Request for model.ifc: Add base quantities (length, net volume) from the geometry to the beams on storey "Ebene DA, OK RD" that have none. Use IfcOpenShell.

First a look at what the model holds.

```python
import ifcopenshell
import ifcopenshell.util.element
import ifcopenshell.util.unit

model = ifcopenshell.open("model.ifc")
print(model.schema)
for unit_type in ("LENGTHUNIT", "AREAUNIT", "VOLUMEUNIT"):
    print(unit_type, ifcopenshell.util.unit.calculate_unit_scale(model, unit_type))
storey = next(s for s in model.by_type("IfcBuildingStorey") if s.Name == "Ebene DA, OK RD")
beams = [e for e in ifcopenshell.util.element.get_decomposition(storey) if e.is_a("IfcBeam")]
for e in sorted(beams, key=lambda e: e.id()):
    print(e.id(), e.is_a(), e.Name, list(ifcopenshell.util.element.get_psets(e, qtos_only=True)), sep=" | ")
```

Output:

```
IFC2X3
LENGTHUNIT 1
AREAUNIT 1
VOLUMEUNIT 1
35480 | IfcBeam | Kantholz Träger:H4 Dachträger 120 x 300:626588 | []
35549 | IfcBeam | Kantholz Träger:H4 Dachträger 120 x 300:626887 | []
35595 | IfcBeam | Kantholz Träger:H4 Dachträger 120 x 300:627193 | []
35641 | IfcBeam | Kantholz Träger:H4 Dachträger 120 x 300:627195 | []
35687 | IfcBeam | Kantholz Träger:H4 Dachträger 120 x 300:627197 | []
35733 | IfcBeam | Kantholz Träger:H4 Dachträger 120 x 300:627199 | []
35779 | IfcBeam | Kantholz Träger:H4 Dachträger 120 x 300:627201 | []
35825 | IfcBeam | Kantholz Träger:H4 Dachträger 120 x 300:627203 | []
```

```python
import ifcopenshell
import ifcopenshell.api.pset
import ifcopenshell.geom
import ifcopenshell.util.element
import ifcopenshell.util.shape
import ifcopenshell.util.unit

model = ifcopenshell.open("model.ifc")
unit_scale = ifcopenshell.util.unit.calculate_unit_scale(model)
volume_scale = ifcopenshell.util.unit.calculate_unit_scale(model, "VOLUMEUNIT")
settings = ifcopenshell.geom.settings()

storey = next(s for s in model.by_type("IfcBuildingStorey") if s.Name == "Ebene DA, OK RD")
beams = [e for e in ifcopenshell.util.element.get_decomposition(storey) if e.is_a("IfcBeam")]

for e in sorted(beams, key=lambda e: e.id()):
    if ifcopenshell.util.element.get_psets(e, qtos_only=True, should_inherit=False):
        continue
    # Geometry comes back in metres, in the element's own axes.
    shape = ifcopenshell.geom.create_shape(settings, e)
    values = {
        "Length": ifcopenshell.util.shape.get_max_xyz(shape.geometry) / unit_scale,
        "NetVolume": ifcopenshell.util.shape.get_volume(shape.geometry) / volume_scale,
    }
    qto = ifcopenshell.api.pset.add_qto(model, product=e, name="BaseQuantities")
    ifcopenshell.api.pset.edit_qto(model, qto=qto, properties=values)
    print(e.id(), {k: round(v, 3) for k, v in values.items()})

model.write("model_edited.ifc")
```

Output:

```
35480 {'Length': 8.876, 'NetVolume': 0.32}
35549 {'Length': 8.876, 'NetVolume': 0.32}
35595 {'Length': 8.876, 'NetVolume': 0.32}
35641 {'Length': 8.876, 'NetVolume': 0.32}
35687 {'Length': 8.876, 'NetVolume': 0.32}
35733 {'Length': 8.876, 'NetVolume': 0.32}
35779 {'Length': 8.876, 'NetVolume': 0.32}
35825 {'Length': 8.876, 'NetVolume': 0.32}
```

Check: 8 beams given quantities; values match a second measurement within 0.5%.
